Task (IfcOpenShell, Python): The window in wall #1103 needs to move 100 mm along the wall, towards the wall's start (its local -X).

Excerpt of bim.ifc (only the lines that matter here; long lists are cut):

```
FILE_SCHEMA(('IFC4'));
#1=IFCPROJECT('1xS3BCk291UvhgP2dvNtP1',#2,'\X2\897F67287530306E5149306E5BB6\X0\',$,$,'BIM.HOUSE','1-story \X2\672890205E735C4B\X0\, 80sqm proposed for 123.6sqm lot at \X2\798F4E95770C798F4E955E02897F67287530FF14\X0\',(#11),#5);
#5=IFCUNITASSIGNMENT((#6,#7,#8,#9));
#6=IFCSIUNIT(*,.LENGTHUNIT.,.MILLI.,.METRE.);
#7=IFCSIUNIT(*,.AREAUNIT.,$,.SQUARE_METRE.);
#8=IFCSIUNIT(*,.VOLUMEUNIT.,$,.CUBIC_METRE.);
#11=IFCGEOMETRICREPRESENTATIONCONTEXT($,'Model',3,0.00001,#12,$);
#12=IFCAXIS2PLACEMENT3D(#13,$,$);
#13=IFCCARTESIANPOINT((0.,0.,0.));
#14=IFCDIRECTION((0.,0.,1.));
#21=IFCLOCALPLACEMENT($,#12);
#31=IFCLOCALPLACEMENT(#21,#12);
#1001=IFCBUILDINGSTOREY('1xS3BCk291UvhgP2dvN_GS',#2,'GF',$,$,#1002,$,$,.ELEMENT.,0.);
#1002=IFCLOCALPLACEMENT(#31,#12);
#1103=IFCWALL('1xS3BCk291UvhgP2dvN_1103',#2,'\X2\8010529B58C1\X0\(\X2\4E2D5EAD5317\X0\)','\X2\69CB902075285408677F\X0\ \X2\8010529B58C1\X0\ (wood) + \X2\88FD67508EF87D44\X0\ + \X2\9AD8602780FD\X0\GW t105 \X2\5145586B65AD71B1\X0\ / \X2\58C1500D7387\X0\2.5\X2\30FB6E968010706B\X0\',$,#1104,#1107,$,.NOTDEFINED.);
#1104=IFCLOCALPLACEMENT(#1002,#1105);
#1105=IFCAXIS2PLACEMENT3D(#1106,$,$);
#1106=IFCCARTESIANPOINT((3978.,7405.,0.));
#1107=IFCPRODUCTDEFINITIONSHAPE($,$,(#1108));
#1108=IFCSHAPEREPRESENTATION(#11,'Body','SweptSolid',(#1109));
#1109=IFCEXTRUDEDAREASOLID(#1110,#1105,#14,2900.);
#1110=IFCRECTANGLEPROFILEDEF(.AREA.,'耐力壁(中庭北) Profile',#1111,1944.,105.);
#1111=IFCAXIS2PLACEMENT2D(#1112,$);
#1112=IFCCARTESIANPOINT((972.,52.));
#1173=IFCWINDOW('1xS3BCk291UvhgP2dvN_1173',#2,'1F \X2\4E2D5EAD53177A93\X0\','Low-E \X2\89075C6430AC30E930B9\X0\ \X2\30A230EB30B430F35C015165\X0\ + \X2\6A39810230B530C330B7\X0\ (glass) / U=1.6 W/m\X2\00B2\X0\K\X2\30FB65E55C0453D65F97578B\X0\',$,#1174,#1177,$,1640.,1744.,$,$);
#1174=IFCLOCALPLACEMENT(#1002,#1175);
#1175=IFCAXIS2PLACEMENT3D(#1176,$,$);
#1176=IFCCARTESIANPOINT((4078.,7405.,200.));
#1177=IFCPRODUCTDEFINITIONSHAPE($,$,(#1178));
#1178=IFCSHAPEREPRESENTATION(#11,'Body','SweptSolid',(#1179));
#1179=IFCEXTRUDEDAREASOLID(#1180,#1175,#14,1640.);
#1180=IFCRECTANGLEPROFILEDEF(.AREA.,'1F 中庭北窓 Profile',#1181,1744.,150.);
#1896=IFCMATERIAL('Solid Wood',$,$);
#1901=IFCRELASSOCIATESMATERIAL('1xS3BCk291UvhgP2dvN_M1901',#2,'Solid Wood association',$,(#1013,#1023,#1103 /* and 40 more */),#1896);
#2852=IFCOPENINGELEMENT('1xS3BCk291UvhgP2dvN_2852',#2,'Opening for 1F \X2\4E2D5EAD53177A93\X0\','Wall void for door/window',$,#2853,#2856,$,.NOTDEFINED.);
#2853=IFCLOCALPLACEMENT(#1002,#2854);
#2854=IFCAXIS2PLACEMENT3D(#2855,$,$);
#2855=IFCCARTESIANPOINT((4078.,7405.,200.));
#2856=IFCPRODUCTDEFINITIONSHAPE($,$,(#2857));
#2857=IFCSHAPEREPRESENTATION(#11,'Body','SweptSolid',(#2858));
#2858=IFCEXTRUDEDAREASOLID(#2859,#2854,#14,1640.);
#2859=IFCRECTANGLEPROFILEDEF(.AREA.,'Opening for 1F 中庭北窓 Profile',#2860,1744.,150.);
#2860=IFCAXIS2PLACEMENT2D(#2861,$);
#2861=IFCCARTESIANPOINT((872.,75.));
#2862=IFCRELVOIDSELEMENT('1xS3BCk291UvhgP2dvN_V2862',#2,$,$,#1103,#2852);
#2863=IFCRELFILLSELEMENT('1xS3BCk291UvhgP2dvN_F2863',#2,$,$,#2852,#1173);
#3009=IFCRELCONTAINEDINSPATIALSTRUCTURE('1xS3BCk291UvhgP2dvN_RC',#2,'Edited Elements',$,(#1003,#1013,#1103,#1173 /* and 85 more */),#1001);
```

```python
import ifcopenshell
import ifcopenshell.api.geometry
import ifcopenshell.util.placement
import ifcopenshell.util.unit

model = ifcopenshell.open("bim.ifc")
unit_scale = ifcopenshell.util.unit.calculate_unit_scale(model)

window = model.by_id(1173)
opening = window.FillsVoids[0].RelatingOpeningElement
wall = opening.VoidsElements[0].RelatingBuildingElement

wall_matrix = ifcopenshell.util.placement.get_local_placement(wall.ObjectPlacement)
shift = wall_matrix[:3, 0] * -0.1 / unit_scale
before = ifcopenshell.util.placement.get_local_placement(window.ObjectPlacement)[:3, 3].copy()

# The window is not placed relative to its opening, so move both.
for product in (opening, window):
    matrix = ifcopenshell.util.placement.get_local_placement(product.ObjectPlacement)
    matrix[:3, 3] += shift
    ifcopenshell.api.geometry.edit_object_placement(model, product=product, matrix=matrix, is_si=False)

after = ifcopenshell.util.placement.get_local_placement(window.ObjectPlacement)[:3, 3]
print("window moved by", (after - before).round(3) + 0.0)

model.write("bim_v2.ifc")
```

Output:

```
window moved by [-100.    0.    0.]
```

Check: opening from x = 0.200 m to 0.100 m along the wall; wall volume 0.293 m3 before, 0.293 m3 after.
